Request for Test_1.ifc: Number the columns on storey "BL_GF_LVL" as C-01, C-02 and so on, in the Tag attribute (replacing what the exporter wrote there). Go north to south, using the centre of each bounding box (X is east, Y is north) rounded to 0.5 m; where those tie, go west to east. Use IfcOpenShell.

First a look at what the model holds.

```python
import ifcopenshell
import ifcopenshell.util.element
import ifcopenshell.util.placement

model = ifcopenshell.open("Test_1.ifc")
print(model.schema)
storey = next(s for s in model.by_type("IfcBuildingStorey") if s.Name == "BL_GF_LVL")
columns = [e for e in ifcopenshell.util.element.get_decomposition(storey) if e.is_a("IfcColumn")]
for e in sorted(columns, key=lambda e: e.id()):
    origin = ifcopenshell.util.placement.get_local_placement(e.ObjectPlacement)[:3, 3]
    print(e.id(), e.Tag, e.Name, origin.round(2) + 0.0, sep=" | ")
```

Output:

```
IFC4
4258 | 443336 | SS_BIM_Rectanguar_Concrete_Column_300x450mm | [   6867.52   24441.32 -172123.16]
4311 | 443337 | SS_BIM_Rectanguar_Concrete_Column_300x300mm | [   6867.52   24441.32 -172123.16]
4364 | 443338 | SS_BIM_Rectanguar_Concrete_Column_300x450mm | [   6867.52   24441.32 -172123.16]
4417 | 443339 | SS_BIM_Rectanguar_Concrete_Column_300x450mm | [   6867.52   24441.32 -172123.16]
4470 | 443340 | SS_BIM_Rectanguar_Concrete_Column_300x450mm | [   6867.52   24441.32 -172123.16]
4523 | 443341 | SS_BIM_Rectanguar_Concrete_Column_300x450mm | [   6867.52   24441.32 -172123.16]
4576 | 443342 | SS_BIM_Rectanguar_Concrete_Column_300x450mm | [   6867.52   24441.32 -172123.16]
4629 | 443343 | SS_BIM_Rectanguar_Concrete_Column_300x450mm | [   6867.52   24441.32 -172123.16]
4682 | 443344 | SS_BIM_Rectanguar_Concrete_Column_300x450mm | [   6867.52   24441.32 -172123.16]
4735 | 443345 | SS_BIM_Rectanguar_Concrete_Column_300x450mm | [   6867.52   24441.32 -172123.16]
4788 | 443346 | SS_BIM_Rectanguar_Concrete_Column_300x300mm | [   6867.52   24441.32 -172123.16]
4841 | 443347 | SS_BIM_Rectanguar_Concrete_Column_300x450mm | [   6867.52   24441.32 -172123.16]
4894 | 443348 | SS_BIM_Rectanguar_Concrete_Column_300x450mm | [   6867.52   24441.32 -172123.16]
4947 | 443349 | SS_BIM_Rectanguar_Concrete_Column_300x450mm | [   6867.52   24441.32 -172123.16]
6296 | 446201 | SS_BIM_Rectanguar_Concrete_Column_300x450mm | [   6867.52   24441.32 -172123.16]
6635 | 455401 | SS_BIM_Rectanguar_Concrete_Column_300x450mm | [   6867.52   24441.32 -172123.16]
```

```python
import ifcopenshell
import ifcopenshell.geom
import ifcopenshell.util.element
import ifcopenshell.util.shape

model = ifcopenshell.open("Test_1.ifc")
settings = ifcopenshell.geom.settings()
settings.set("use-world-coords", True)


def centre(element):
    shape = ifcopenshell.geom.create_shape(settings, element)
    return ifcopenshell.util.shape.get_bbox_centroid(shape.geometry)


storey = next(s for s in model.by_type("IfcBuildingStorey") if s.Name == "BL_GF_LVL")
columns = [e for e in ifcopenshell.util.element.get_decomposition(storey) if e.is_a("IfcColumn")]

# Insertion points can sit at a corner or the storey origin, so sort by the geometry (in metres).
centres = {e: centre(e) for e in columns}
columns.sort(key=lambda e: (-round(centres[e][1] / 0.5), centres[e][0]))

for i, e in enumerate(columns, start=1):
    number = f"C-{i:02d}"
    e.Tag = number
    print(e.id(), number)

model.write("Test_1_v2.ifc")
```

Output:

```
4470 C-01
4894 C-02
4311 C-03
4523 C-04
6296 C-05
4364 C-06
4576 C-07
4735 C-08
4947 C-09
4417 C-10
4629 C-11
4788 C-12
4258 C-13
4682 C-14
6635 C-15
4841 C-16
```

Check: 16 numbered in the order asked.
